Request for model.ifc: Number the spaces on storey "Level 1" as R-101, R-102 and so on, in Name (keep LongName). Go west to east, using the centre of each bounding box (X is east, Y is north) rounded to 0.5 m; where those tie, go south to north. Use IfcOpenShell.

First a look at what the model holds.

```python
import ifcopenshell
import ifcopenshell.util.element
import ifcopenshell.util.placement

model = ifcopenshell.open("model.ifc")
print(model.schema)
storey = next(s for s in model.by_type("IfcBuildingStorey") if s.Name == "Level 1")
spaces = [e for e in ifcopenshell.util.element.get_decomposition(storey) if e.is_a("IfcSpace")]
for e in sorted(spaces, key=lambda e: e.id()):
    origin = ifcopenshell.util.placement.get_local_placement(e.ObjectPlacement)[:3, 3]
    print(e.id(), e.Name, e.LongName, origin.round(2) + 0.0, sep=" | ")
```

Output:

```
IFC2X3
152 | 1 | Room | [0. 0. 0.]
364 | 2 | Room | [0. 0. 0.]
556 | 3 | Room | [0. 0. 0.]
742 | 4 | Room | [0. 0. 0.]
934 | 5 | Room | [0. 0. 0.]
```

```python
import ifcopenshell
import ifcopenshell.geom
import ifcopenshell.util.element
import ifcopenshell.util.shape

model = ifcopenshell.open("model.ifc")
settings = ifcopenshell.geom.settings()
settings.set("use-world-coords", True)


def centre(element):
    shape = ifcopenshell.geom.create_shape(settings, element)
    return ifcopenshell.util.shape.get_bbox_centroid(shape.geometry)


storey = next(s for s in model.by_type("IfcBuildingStorey") if s.Name == "Level 1")
spaces = [e for e in ifcopenshell.util.element.get_decomposition(storey) if e.is_a("IfcSpace")]

# Insertion points can sit at a corner or the storey origin, so sort by the geometry (in metres).
centres = {e: centre(e) for e in spaces}
spaces.sort(key=lambda e: (round(centres[e][0] / 0.5), centres[e][1]))

for i, e in enumerate(spaces, start=1):
    number = f"R-1{i:02d}"
    e.Name = number
    print(e.id(), number)

model.write("model_v2.ifc")
```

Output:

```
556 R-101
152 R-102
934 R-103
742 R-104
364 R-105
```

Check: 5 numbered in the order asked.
